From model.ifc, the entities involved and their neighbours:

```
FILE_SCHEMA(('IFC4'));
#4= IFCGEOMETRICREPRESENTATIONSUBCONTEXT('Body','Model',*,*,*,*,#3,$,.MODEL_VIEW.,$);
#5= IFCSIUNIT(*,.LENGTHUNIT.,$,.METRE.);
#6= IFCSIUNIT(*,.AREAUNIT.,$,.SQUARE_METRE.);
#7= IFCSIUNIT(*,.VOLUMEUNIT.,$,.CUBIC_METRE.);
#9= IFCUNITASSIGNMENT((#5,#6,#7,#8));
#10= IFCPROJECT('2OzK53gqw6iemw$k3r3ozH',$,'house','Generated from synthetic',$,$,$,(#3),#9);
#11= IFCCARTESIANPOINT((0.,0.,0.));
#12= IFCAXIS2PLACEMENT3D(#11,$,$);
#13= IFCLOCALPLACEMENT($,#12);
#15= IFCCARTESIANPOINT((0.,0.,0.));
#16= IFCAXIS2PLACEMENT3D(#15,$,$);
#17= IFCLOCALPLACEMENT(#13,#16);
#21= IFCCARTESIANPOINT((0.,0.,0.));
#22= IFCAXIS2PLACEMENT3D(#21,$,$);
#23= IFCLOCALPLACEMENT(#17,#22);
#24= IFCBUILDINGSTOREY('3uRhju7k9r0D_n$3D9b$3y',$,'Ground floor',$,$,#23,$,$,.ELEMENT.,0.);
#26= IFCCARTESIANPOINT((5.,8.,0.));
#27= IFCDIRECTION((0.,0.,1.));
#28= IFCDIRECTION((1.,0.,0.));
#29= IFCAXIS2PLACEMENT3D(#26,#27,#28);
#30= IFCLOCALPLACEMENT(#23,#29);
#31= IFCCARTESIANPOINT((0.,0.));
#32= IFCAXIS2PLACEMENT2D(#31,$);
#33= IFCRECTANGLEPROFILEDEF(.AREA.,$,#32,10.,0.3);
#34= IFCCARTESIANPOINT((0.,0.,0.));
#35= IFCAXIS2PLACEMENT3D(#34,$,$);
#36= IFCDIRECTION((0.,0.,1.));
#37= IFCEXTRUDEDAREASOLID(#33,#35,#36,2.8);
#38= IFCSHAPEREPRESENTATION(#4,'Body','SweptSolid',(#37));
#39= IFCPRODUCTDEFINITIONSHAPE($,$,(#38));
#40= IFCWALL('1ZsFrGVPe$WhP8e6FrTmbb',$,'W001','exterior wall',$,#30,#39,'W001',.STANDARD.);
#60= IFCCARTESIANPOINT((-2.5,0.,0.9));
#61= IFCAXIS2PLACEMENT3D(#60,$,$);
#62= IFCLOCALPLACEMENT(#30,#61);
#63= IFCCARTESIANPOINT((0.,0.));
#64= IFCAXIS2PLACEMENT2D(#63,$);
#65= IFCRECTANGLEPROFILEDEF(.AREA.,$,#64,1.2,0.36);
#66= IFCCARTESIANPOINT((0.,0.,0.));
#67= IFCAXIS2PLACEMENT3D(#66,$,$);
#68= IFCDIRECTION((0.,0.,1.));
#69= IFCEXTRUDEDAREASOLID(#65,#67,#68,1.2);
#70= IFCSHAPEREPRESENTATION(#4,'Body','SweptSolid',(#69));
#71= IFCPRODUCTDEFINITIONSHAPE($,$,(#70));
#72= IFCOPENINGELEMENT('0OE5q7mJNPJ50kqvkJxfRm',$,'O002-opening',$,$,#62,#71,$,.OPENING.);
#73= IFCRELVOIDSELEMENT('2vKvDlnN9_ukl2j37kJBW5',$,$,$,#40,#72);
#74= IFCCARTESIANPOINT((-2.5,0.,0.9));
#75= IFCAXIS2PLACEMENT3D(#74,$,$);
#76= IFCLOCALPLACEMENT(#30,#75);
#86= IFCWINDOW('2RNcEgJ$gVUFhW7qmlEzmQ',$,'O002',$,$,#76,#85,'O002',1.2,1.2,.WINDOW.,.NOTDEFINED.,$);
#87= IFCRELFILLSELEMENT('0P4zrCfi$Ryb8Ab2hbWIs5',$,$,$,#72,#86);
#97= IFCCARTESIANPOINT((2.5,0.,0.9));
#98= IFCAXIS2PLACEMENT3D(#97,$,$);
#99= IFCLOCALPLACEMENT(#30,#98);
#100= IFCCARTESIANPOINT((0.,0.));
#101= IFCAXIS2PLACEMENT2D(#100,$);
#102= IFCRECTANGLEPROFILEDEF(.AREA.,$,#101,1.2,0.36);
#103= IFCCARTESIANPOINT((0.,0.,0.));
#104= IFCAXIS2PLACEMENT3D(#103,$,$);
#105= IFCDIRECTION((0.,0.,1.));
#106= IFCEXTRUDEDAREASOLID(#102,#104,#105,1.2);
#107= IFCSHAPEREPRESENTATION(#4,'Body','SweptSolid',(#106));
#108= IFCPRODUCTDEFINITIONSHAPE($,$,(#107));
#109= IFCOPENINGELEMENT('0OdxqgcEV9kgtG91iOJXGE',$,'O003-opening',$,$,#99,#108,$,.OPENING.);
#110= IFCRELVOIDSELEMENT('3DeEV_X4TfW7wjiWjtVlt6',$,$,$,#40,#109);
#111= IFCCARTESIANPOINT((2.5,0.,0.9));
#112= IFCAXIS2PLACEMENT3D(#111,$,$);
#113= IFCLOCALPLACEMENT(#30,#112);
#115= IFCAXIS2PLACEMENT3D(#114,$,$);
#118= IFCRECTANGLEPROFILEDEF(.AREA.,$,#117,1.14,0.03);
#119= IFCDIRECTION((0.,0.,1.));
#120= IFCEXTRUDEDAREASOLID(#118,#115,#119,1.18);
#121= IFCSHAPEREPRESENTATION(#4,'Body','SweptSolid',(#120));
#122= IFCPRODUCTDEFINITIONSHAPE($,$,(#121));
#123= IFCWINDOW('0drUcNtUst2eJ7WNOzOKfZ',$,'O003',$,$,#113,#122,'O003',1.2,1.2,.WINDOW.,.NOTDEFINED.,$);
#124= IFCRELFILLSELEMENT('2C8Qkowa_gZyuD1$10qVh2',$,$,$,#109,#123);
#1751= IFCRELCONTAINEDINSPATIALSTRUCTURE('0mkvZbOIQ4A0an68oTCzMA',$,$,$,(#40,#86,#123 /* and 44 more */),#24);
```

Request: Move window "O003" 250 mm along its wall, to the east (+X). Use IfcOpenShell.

```python
import ifcopenshell
import ifcopenshell.api.geometry
import ifcopenshell.util.placement
import ifcopenshell.util.unit

model = ifcopenshell.open("model.ifc")
unit_scale = ifcopenshell.util.unit.calculate_unit_scale(model)

window = model.by_guid("0drUcNtUst2eJ7WNOzOKfZ")
opening = window.FillsVoids[0].RelatingOpeningElement
wall = opening.VoidsElements[0].RelatingBuildingElement

wall_matrix = ifcopenshell.util.placement.get_local_placement(wall.ObjectPlacement)
shift = wall_matrix[:3, 0] * 0.25 / unit_scale
before = ifcopenshell.util.placement.get_local_placement(window.ObjectPlacement)[:3, 3].copy()

# The window is not placed relative to its opening, so move both.
for product in (opening, window):
    matrix = ifcopenshell.util.placement.get_local_placement(product.ObjectPlacement)
    matrix[:3, 3] += shift
    ifcopenshell.api.geometry.edit_object_placement(model, product=product, matrix=matrix, is_si=False)

after = ifcopenshell.util.placement.get_local_placement(window.ObjectPlacement)[:3, 3]
print("window moved by", (after - before).round(3) + 0.0)

model.write("model_v2.ifc")
```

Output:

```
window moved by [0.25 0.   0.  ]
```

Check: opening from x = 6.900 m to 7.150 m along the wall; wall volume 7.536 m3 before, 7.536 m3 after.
